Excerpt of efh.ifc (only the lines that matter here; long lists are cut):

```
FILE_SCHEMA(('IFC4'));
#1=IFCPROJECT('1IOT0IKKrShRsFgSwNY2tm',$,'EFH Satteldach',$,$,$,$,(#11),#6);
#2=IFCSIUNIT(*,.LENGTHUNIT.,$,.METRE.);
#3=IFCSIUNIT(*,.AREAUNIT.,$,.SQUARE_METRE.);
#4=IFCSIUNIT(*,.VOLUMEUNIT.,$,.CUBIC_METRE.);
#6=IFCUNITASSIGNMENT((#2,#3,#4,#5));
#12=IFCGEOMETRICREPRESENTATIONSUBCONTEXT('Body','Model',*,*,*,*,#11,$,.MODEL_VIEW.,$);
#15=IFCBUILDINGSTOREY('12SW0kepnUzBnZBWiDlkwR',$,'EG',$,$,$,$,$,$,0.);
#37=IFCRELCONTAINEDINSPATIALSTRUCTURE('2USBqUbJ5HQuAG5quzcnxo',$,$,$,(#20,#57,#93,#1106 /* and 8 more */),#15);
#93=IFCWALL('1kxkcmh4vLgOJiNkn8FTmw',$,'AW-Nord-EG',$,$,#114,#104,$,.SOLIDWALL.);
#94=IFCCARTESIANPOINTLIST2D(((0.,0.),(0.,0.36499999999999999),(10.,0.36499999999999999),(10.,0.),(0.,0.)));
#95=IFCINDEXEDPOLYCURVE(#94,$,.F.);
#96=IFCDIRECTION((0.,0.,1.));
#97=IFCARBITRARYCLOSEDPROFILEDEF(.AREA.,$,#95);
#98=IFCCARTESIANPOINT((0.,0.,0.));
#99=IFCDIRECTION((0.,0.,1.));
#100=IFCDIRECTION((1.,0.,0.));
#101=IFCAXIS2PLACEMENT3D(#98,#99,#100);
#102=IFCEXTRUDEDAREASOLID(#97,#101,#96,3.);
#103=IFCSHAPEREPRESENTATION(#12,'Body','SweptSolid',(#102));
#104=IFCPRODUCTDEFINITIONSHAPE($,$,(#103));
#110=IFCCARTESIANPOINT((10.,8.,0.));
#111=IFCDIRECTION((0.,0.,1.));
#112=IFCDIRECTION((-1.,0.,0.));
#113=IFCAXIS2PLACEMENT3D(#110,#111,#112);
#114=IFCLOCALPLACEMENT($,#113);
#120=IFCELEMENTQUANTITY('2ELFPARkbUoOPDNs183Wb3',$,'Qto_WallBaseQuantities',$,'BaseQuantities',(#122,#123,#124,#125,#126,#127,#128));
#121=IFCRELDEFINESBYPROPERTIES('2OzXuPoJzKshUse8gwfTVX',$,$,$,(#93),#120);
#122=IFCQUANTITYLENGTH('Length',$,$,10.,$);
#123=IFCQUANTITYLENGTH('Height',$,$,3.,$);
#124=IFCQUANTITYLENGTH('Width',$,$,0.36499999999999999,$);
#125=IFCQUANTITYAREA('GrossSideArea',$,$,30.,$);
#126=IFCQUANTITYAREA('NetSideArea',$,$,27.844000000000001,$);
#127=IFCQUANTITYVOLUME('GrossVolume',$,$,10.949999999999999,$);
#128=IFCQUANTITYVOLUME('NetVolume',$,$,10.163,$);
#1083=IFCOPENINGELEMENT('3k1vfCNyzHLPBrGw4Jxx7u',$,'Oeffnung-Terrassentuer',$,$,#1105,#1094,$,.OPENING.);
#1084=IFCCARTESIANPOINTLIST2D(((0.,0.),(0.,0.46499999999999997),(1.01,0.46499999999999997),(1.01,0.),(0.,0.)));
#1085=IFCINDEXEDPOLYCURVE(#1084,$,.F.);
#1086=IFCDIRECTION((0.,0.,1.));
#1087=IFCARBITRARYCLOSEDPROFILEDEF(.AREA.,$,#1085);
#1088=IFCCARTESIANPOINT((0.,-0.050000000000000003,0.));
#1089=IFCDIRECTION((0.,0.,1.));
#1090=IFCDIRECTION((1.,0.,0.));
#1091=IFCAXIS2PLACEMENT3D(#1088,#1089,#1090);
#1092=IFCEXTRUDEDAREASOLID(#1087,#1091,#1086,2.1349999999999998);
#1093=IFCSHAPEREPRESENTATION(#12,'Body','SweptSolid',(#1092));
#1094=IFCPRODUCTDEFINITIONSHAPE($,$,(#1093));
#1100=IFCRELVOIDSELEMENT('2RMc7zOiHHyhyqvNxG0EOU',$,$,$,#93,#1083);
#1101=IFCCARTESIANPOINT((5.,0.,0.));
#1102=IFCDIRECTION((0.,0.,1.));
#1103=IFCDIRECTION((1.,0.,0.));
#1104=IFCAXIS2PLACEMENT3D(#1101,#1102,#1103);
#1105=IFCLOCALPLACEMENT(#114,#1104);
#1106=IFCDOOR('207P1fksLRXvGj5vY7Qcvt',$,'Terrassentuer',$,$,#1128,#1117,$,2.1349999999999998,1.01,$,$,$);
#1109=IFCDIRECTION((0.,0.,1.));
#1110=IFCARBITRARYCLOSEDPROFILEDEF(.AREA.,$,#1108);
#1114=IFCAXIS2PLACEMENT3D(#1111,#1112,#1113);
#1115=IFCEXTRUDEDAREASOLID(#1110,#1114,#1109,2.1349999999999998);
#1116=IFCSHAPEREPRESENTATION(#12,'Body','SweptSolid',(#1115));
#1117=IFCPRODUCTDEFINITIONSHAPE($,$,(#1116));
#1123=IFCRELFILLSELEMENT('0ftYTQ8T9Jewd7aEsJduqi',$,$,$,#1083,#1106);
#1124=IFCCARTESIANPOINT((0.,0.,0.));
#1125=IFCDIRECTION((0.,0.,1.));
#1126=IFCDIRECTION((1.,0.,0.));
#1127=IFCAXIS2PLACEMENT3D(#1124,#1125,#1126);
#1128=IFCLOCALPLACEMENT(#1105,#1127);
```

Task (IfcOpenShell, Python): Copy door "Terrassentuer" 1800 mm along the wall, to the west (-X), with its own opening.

```python
import ifcopenshell
import ifcopenshell.api.feature
import ifcopenshell.api.geometry
import ifcopenshell.api.pset
import ifcopenshell.api.root
import ifcopenshell.geom
import ifcopenshell.util.element
import ifcopenshell.util.placement
import ifcopenshell.util.shape
import ifcopenshell.util.unit

model = ifcopenshell.open("efh.ifc")
unit_scale = ifcopenshell.util.unit.calculate_unit_scale(model)
area_scale = ifcopenshell.util.unit.calculate_unit_scale(model, "AREAUNIT")
volume_scale = ifcopenshell.util.unit.calculate_unit_scale(model, "VOLUMEUNIT")
settings = ifcopenshell.geom.settings()


def volume(element):
    """Net volume in cubic metres, openings subtracted."""
    shape = ifcopenshell.geom.create_shape(settings, element)
    return ifcopenshell.util.shape.get_volume(shape.geometry)


door = model.by_guid("207P1fksLRXvGj5vY7Qcvt")
opening = door.FillsVoids[0].RelatingOpeningElement
wall = opening.VoidsElements[0].RelatingBuildingElement
before = volume(wall)
shift = ifcopenshell.util.placement.get_local_placement(wall.ObjectPlacement)[:3, 0] * 1.8 / unit_scale

# copy_class copies the void relationship, type, container and properties, but no geometry.
new_opening = ifcopenshell.api.root.copy_class(model, product=opening)
new_opening.Representation = ifcopenshell.util.element.copy_deep(
    model, opening.Representation, exclude=["IfcGeometricRepresentationContext", "IfcRepresentationMap"]
)
new_door = ifcopenshell.api.root.copy_class(model, product=door)
new_door.Representation = ifcopenshell.util.element.copy_deep(
    model, door.Representation, exclude=["IfcGeometricRepresentationContext", "IfcRepresentationMap"]
)
ifcopenshell.api.feature.add_filling(model, opening=new_opening, element=new_door)

for old, new in ((opening, new_opening), (door, new_door)):
    matrix = ifcopenshell.util.placement.get_local_placement(old.ObjectPlacement)
    matrix[:3, 3] += shift
    ifcopenshell.api.geometry.edit_object_placement(model, product=new, matrix=matrix, is_si=False)

after = volume(wall)
thickness = 0.365  # wall thickness in metres

# Update the wall's stored quantities.
qto = model.by_id(ifcopenshell.util.element.get_pset(wall, "Qto_WallBaseQuantities", should_inherit=False)["id"])
ifcopenshell.api.pset.edit_qto(model, qto=qto, properties={
    "NetSideArea": after / thickness / area_scale,
    "NetVolume": after / volume_scale,
})

print(f"wall volume {before:.3f} -> {after:.3f} m3")

model.write("efh_edited.ifc")
```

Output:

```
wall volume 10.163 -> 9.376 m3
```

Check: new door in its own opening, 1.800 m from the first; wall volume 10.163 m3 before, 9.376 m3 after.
